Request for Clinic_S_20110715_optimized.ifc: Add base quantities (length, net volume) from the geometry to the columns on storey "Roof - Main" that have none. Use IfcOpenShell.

First a look at what the model holds.

```python
import ifcopenshell
import ifcopenshell.util.element
import ifcopenshell.util.unit

model = ifcopenshell.open("Clinic_S_20110715_optimized.ifc")
print(model.schema)
for unit_type in ("LENGTHUNIT", "AREAUNIT", "VOLUMEUNIT"):
    print(unit_type, ifcopenshell.util.unit.calculate_unit_scale(model, unit_type))
storey = next(s for s in model.by_type("IfcBuildingStorey") if s.Name == "Roof - Main")
columns = [e for e in ifcopenshell.util.element.get_decomposition(storey) if e.is_a("IfcColumn")]
for e in sorted(columns, key=lambda e: e.id()):
    print(e.id(), e.is_a(), e.Name, list(ifcopenshell.util.element.get_psets(e, qtos_only=True)), sep=" | ")
```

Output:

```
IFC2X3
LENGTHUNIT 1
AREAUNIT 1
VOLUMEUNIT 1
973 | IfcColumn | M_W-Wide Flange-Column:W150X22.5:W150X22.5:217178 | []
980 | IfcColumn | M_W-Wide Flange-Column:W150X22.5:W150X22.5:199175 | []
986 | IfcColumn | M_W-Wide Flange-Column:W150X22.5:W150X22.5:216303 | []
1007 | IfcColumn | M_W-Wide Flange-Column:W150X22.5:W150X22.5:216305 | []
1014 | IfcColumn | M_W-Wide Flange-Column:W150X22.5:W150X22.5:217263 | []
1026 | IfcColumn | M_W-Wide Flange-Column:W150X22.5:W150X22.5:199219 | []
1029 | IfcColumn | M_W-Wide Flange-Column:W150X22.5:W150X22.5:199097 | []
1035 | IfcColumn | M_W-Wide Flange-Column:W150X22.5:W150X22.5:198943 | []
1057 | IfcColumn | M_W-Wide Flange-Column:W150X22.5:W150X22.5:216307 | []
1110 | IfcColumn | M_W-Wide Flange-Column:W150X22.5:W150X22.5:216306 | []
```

```python
import ifcopenshell
import ifcopenshell.api.pset
import ifcopenshell.geom
import ifcopenshell.util.element
import ifcopenshell.util.shape
import ifcopenshell.util.unit

model = ifcopenshell.open("Clinic_S_20110715_optimized.ifc")
unit_scale = ifcopenshell.util.unit.calculate_unit_scale(model)
volume_scale = ifcopenshell.util.unit.calculate_unit_scale(model, "VOLUMEUNIT")
settings = ifcopenshell.geom.settings()

storey = next(s for s in model.by_type("IfcBuildingStorey") if s.Name == "Roof - Main")
columns = [e for e in ifcopenshell.util.element.get_decomposition(storey) if e.is_a("IfcColumn")]

for e in sorted(columns, key=lambda e: e.id()):
    if ifcopenshell.util.element.get_psets(e, qtos_only=True, should_inherit=False):
        continue
    # Geometry comes back in metres, in the element's own axes.
    shape = ifcopenshell.geom.create_shape(settings, e)
    values = {
        "Length": ifcopenshell.util.shape.get_z(shape.geometry) / unit_scale,
        "NetVolume": ifcopenshell.util.shape.get_volume(shape.geometry) / volume_scale,
    }
    qto = ifcopenshell.api.pset.add_qto(model, product=e, name="BaseQuantities")
    ifcopenshell.api.pset.edit_qto(model, qto=qto, properties=values)
    print(e.id(), {k: round(v, 3) for k, v in values.items()})

model.write("Clinic_S_20110715_optimized_rev.ifc")
```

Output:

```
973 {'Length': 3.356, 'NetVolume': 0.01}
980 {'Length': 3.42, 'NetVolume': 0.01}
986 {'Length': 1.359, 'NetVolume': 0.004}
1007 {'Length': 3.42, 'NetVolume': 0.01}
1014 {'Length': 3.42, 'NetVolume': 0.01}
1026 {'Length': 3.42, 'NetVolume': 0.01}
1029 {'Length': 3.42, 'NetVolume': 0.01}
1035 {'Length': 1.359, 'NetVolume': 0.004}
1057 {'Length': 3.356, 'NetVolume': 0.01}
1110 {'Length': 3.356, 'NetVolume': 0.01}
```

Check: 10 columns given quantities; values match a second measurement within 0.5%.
